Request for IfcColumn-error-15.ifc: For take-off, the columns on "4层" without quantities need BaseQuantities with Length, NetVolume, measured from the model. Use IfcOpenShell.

First a look at what the model holds.

```python
import ifcopenshell
import ifcopenshell.util.element
import ifcopenshell.util.unit

model = ifcopenshell.open("IfcColumn-error-15.ifc")
print(model.schema)
for unit_type in ("LENGTHUNIT", "AREAUNIT", "VOLUMEUNIT"):
    print(unit_type, ifcopenshell.util.unit.calculate_unit_scale(model, unit_type))
storey = next(s for s in model.by_type("IfcBuildingStorey") if s.Name == "4层")
columns = [e for e in ifcopenshell.util.element.get_decomposition(storey) if e.is_a("IfcColumn")]
for e in sorted(columns, key=lambda e: e.id()):
    print(e.id(), e.is_a(), e.Name, list(ifcopenshell.util.element.get_psets(e, qtos_only=True)), sep=" | ")
```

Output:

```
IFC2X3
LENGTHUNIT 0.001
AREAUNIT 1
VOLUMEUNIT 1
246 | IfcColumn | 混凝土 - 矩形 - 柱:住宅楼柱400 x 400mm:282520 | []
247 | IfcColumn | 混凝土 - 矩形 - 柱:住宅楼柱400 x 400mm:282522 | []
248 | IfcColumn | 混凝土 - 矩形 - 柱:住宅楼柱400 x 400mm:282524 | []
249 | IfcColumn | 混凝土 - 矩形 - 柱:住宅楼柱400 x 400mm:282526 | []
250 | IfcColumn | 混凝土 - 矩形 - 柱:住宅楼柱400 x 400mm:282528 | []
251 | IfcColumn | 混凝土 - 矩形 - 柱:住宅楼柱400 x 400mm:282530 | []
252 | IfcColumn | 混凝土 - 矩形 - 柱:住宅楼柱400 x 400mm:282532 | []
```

```python
import ifcopenshell
import ifcopenshell.api.pset
import ifcopenshell.geom
import ifcopenshell.util.element
import ifcopenshell.util.shape
import ifcopenshell.util.unit

model = ifcopenshell.open("IfcColumn-error-15.ifc")
unit_scale = ifcopenshell.util.unit.calculate_unit_scale(model)
volume_scale = ifcopenshell.util.unit.calculate_unit_scale(model, "VOLUMEUNIT")
settings = ifcopenshell.geom.settings()

storey = next(s for s in model.by_type("IfcBuildingStorey") if s.Name == "4层")
columns = [e for e in ifcopenshell.util.element.get_decomposition(storey) if e.is_a("IfcColumn")]

for e in sorted(columns, key=lambda e: e.id()):
    if ifcopenshell.util.element.get_psets(e, qtos_only=True, should_inherit=False):
        continue
    # Geometry comes back in metres, in the element's own axes.
    shape = ifcopenshell.geom.create_shape(settings, e)
    values = {
        "Length": ifcopenshell.util.shape.get_z(shape.geometry) / unit_scale,
        "NetVolume": ifcopenshell.util.shape.get_volume(shape.geometry) / volume_scale,
    }
    qto = ifcopenshell.api.pset.add_qto(model, product=e, name="BaseQuantities")
    ifcopenshell.api.pset.edit_qto(model, qto=qto, properties=values)
    print(e.id(), {k: round(v, 3) for k, v in values.items()})

model.write("IfcColumn-error-15_rev.ifc")
```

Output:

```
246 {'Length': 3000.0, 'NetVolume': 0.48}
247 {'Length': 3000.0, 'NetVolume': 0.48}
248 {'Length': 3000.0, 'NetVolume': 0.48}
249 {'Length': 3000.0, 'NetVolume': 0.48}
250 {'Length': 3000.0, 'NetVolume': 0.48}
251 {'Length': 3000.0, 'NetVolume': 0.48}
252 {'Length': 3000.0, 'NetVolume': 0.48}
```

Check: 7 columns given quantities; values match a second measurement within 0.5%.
